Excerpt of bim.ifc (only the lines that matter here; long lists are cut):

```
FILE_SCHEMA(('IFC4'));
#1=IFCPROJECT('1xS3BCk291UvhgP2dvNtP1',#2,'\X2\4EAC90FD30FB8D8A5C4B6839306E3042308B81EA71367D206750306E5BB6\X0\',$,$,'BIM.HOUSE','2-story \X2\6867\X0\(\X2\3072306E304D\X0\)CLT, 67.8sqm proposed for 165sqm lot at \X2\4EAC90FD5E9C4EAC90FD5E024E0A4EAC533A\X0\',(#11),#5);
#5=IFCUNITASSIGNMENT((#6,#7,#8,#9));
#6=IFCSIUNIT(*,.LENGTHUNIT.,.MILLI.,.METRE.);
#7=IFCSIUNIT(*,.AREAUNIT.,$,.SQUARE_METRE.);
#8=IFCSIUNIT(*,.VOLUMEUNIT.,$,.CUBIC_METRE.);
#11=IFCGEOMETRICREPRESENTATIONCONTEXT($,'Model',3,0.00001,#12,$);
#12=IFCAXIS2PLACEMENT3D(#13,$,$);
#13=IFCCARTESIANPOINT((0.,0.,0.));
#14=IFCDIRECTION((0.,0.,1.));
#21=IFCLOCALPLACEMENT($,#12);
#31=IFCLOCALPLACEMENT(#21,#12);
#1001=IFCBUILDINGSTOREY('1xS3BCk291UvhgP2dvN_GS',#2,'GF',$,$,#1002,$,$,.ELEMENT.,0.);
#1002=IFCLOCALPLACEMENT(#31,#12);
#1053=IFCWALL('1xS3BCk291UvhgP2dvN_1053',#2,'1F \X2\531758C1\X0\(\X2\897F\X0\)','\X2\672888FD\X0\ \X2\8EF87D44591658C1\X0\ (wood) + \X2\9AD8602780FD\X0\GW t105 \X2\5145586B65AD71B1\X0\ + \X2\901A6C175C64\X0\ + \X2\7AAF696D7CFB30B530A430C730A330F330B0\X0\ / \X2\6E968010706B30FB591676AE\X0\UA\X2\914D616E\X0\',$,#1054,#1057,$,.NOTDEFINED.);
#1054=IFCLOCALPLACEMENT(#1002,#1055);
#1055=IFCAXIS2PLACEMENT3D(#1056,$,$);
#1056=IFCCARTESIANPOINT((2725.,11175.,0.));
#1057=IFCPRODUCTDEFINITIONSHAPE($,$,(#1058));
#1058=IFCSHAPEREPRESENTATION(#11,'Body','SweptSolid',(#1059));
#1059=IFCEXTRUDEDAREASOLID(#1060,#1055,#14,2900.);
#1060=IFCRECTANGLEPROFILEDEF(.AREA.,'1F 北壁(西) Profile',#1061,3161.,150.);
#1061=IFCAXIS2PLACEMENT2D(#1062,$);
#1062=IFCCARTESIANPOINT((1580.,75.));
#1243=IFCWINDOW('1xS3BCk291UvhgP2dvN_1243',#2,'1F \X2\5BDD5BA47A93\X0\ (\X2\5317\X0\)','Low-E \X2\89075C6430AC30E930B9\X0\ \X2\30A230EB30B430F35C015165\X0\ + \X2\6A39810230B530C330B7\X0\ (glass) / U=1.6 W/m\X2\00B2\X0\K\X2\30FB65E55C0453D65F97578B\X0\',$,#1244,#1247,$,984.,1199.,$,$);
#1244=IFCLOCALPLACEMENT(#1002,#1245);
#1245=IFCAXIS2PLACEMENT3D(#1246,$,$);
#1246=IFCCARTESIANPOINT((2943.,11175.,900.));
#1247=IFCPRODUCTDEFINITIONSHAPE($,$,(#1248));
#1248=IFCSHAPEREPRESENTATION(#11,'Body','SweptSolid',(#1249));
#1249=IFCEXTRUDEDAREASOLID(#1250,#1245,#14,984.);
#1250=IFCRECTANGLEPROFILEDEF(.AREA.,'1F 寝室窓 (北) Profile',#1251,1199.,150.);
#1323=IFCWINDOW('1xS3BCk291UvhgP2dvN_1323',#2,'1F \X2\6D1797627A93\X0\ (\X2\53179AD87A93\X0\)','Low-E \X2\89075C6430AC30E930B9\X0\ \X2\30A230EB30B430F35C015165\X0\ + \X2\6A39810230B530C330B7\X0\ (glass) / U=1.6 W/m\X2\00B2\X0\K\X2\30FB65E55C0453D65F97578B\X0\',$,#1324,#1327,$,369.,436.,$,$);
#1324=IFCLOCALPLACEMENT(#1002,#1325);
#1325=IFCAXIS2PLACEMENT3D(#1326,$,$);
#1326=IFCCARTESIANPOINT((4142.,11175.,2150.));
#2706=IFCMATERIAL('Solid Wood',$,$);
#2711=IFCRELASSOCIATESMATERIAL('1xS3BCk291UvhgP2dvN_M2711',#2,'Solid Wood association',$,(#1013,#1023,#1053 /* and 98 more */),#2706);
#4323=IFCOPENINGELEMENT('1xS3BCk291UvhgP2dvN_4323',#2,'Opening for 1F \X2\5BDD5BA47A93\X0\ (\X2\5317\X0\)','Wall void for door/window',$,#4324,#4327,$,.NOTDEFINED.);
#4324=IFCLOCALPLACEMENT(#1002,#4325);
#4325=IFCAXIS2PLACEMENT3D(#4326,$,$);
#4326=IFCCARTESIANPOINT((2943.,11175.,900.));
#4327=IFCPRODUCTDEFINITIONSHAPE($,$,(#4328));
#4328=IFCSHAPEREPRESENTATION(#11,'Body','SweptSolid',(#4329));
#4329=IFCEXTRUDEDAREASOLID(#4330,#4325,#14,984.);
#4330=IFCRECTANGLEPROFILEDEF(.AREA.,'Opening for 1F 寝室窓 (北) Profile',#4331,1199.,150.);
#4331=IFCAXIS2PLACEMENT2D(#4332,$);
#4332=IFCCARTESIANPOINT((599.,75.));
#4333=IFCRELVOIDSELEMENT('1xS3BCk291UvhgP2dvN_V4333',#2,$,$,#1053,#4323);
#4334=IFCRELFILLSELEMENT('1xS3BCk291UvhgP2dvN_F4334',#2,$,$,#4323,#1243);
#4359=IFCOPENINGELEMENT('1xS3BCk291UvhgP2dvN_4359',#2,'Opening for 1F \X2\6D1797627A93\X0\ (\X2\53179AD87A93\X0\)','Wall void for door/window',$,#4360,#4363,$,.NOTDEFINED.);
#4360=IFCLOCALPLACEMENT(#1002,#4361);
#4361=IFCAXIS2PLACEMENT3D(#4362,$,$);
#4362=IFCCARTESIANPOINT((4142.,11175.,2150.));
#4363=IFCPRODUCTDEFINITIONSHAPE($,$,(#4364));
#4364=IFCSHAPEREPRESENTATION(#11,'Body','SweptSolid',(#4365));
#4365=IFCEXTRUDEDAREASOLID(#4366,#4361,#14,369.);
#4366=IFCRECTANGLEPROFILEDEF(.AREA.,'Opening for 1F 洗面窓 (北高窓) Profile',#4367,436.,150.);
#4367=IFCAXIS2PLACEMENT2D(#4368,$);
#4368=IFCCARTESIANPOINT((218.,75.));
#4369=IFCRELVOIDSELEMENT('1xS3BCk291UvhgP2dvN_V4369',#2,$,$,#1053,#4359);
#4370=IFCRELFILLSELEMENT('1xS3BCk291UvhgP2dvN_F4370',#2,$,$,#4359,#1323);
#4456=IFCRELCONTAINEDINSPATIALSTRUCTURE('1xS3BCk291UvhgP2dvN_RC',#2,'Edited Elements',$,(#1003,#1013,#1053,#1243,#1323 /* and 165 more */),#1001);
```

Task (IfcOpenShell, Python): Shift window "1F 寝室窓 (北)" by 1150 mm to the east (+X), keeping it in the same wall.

```python
import ifcopenshell
import ifcopenshell.api.geometry
import ifcopenshell.util.placement
import ifcopenshell.util.unit

model = ifcopenshell.open("bim.ifc")
unit_scale = ifcopenshell.util.unit.calculate_unit_scale(model)

window = model.by_guid("1xS3BCk291UvhgP2dvN_1243")
opening = window.FillsVoids[0].RelatingOpeningElement
wall = opening.VoidsElements[0].RelatingBuildingElement

wall_matrix = ifcopenshell.util.placement.get_local_placement(wall.ObjectPlacement)
shift = wall_matrix[:3, 0] * 1.15 / unit_scale
before = ifcopenshell.util.placement.get_local_placement(window.ObjectPlacement)[:3, 3].copy()

# The window is not placed relative to its opening, so move both.
for product in (opening, window):
    matrix = ifcopenshell.util.placement.get_local_placement(product.ObjectPlacement)
    matrix[:3, 3] += shift
    ifcopenshell.api.geometry.edit_object_placement(model, product=product, matrix=matrix, is_si=False)

after = ifcopenshell.util.placement.get_local_placement(window.ObjectPlacement)[:3, 3]
print("window moved by", (after - before).round(3) + 0.0)

model.write("bim_rev.ifc")
```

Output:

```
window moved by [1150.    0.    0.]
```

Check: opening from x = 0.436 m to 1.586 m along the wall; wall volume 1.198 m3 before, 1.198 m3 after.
